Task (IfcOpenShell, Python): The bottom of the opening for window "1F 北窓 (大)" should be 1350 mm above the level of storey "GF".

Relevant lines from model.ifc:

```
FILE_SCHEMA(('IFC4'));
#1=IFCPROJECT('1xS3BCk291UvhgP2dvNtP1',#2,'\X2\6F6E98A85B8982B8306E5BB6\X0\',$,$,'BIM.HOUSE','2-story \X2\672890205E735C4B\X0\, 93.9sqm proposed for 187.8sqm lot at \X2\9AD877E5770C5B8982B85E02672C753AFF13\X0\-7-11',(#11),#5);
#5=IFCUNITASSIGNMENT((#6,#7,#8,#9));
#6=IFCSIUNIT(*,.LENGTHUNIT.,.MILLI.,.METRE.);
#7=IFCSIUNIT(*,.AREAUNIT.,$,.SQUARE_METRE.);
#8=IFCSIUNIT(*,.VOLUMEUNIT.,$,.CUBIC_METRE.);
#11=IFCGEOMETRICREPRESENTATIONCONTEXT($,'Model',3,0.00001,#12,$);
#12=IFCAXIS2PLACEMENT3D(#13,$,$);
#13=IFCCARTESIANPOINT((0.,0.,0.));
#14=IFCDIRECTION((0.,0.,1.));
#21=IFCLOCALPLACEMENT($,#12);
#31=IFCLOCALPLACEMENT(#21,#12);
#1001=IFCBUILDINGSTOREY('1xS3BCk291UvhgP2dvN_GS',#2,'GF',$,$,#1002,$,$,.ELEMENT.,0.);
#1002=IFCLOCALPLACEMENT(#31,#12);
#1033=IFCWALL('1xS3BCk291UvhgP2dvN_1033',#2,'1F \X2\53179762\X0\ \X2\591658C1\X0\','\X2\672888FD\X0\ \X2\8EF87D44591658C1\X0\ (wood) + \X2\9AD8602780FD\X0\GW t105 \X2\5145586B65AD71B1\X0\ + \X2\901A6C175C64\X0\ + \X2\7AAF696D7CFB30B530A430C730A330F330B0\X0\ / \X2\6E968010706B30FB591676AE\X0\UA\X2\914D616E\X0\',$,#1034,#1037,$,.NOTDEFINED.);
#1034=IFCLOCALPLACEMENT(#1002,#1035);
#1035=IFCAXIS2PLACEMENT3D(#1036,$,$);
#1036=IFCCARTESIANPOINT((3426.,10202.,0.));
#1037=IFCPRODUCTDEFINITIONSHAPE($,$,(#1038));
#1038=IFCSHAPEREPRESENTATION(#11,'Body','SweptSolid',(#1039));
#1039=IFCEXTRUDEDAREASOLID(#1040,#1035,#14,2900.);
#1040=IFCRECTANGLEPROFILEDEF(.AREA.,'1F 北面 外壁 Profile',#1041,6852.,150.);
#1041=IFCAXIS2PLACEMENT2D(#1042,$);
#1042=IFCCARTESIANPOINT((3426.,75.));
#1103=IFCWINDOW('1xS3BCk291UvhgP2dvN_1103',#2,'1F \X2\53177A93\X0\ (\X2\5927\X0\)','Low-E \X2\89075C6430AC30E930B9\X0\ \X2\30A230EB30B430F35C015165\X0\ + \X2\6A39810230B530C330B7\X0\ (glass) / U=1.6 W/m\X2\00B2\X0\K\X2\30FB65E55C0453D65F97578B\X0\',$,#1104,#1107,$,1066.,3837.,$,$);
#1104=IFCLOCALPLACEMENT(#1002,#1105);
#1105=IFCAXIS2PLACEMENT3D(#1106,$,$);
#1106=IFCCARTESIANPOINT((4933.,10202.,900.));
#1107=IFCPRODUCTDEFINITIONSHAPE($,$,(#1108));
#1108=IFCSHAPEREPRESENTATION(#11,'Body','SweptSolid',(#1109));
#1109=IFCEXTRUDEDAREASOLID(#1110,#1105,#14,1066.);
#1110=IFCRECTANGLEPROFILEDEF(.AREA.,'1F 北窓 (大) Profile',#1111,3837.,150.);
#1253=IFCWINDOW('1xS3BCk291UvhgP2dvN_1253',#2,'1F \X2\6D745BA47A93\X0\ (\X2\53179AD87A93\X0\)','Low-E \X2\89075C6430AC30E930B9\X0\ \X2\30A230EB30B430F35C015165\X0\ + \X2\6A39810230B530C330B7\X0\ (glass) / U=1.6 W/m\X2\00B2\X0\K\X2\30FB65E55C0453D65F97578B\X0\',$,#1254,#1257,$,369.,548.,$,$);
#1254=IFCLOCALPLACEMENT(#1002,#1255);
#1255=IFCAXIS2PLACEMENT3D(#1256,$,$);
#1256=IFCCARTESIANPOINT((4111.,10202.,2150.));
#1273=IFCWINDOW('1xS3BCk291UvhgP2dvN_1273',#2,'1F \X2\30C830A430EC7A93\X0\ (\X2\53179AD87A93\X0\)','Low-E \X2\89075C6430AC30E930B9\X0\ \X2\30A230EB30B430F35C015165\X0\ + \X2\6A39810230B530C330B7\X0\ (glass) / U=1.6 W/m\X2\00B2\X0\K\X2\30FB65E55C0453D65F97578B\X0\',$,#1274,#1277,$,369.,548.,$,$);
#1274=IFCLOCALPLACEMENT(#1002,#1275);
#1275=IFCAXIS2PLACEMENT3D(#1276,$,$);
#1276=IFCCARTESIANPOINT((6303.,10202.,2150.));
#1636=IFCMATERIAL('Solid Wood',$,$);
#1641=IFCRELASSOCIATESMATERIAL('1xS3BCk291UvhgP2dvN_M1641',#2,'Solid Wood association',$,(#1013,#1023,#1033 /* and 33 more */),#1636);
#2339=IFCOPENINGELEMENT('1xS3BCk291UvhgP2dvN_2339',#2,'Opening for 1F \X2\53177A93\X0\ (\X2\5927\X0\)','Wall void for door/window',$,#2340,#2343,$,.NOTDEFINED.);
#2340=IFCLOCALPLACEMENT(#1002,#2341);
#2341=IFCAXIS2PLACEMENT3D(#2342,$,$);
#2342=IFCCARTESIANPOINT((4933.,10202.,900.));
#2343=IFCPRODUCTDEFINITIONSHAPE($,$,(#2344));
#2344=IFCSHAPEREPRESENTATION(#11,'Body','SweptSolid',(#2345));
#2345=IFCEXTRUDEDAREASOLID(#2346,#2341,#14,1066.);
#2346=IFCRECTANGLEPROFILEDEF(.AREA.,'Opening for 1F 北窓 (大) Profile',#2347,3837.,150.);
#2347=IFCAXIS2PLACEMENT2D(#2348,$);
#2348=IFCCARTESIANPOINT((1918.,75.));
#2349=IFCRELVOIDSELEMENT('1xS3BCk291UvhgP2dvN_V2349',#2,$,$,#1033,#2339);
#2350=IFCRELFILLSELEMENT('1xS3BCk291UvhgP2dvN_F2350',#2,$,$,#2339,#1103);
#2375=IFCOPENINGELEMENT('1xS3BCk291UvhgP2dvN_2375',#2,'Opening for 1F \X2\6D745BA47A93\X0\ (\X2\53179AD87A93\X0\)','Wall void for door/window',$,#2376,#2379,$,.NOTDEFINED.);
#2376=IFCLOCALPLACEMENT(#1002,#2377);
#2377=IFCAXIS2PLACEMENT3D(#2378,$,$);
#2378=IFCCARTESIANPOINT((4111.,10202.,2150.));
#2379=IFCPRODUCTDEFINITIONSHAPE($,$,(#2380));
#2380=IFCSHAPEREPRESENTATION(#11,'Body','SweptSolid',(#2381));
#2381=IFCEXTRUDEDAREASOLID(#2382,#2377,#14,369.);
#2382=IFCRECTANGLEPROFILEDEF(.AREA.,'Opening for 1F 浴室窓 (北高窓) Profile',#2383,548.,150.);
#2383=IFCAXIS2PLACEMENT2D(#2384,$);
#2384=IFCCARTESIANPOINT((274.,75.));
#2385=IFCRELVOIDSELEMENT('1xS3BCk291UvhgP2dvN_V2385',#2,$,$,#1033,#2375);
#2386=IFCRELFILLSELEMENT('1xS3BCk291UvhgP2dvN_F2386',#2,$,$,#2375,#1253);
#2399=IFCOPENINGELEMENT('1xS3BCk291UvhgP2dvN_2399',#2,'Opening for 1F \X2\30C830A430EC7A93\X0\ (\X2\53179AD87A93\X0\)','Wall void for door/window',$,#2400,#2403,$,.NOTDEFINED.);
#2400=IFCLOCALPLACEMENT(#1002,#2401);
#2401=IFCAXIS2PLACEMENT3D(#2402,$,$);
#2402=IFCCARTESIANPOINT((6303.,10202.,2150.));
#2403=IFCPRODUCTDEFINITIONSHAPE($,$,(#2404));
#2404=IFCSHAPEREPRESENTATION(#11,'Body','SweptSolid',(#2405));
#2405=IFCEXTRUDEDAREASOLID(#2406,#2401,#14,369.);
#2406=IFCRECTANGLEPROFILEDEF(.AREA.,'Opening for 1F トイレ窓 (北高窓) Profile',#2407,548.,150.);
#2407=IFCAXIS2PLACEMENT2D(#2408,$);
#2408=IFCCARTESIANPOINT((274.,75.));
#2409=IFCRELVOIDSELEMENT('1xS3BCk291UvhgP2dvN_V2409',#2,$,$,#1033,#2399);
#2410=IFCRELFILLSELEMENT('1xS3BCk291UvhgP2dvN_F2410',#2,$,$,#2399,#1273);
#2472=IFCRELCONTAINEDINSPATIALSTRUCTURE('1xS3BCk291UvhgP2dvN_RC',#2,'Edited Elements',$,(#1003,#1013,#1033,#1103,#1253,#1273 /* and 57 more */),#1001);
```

```python
import numpy as np
import ifcopenshell
import ifcopenshell.api.geometry
import ifcopenshell.geom
import ifcopenshell.util.element
import ifcopenshell.util.placement
import ifcopenshell.util.shape
import ifcopenshell.util.unit

model = ifcopenshell.open("model.ifc")
unit_scale = ifcopenshell.util.unit.calculate_unit_scale(model)

window = model.by_guid("1xS3BCk291UvhgP2dvN_1103")
opening = window.FillsVoids[0].RelatingOpeningElement
storey = ifcopenshell.util.element.get_container(window, ifc_class="IfcBuildingStorey")
level = ifcopenshell.util.placement.get_local_placement(storey.ObjectPlacement)[2, 3]

# The opening's origin need not be at the sill, so measure its lowest point.
shape = ifcopenshell.geom.create_shape(ifcopenshell.geom.settings(), opening)
bottom = ifcopenshell.util.shape.get_shape_bottom_elevation(shape, shape.geometry) / unit_scale
dz = level + 1.35 / unit_scale - bottom

shift = np.array([0.0, 0.0, dz])
# The window is not placed relative to its opening, so move both.
for product in (opening, window):
    matrix = ifcopenshell.util.placement.get_local_placement(product.ObjectPlacement)
    matrix[:3, 3] += shift
    ifcopenshell.api.geometry.edit_object_placement(model, product=product, matrix=matrix, is_si=False)

print(f"moved by {dz * unit_scale:+.3f} m")

model.write("model_v2.ifc")
```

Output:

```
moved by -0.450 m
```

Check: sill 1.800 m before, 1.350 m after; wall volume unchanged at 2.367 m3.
